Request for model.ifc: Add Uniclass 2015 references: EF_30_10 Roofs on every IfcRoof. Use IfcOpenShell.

First a look at what the model holds.

```python
import ifcopenshell

model = ifcopenshell.open("model.ifc")
print(model.schema)
print("classifications:", [c.Name for c in model.by_type("IfcClassification")])
for ifc_class in ("IfcDoor", "IfcRoof", "IfcStair", "IfcWall", "IfcWindow"):
    print(ifc_class, len(model.by_type(ifc_class)))
```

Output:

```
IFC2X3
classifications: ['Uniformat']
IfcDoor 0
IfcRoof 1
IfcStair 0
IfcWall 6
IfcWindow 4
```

```python
import ifcopenshell
import ifcopenshell.api.classification

model = ifcopenshell.open("model.ifc")

# IFC2X3 requires Source and Edition and has no link from the project to the system.
system = model.create_entity("IfcClassification", Source="NBS", Edition="2015", Name="Uniclass 2015")

codes = {
    "IfcRoof": ("EF_30_10", "Roofs"),
}
for ifc_class, (code, name) in codes.items():
    products = model.by_type(ifc_class)
    ifcopenshell.api.classification.add_reference(
        model, products=products, classification=system, identification=code, name=name
    )
    print(code, len(products))

model.write("model_updated.ifc")
```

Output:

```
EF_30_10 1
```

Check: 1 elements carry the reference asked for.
